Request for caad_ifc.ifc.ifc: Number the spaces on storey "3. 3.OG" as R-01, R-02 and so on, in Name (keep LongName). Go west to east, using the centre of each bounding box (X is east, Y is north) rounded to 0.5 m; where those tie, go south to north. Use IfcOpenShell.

First a look at what the model holds.

```python
import ifcopenshell
import ifcopenshell.util.element
import ifcopenshell.util.placement

model = ifcopenshell.open("caad_ifc.ifc.ifc")
print(model.schema)
storey = next(s for s in model.by_type("IfcBuildingStorey") if s.Name == "3. 3.OG")
spaces = [e for e in ifcopenshell.util.element.get_decomposition(storey) if e.is_a("IfcSpace")]
for e in sorted(spaces, key=lambda e: e.id()):
    origin = ifcopenshell.util.placement.get_local_placement(e.ObjectPlacement)[:3, 3]
    print(e.id(), e.Name, e.LongName, origin.round(2) + 0.0, sep=" | ")
```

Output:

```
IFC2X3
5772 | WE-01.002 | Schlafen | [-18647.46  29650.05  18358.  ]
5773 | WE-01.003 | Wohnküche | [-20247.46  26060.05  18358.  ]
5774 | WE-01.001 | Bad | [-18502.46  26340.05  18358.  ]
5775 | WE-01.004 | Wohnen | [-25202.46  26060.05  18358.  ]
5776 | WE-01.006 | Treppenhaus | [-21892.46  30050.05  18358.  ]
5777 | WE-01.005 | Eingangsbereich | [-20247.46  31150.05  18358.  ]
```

```python
import ifcopenshell
import ifcopenshell.geom
import ifcopenshell.util.element
import ifcopenshell.util.shape

model = ifcopenshell.open("caad_ifc.ifc.ifc")
settings = ifcopenshell.geom.settings()
settings.set("use-world-coords", True)


def centre(element):
    shape = ifcopenshell.geom.create_shape(settings, element)
    return ifcopenshell.util.shape.get_bbox_centroid(shape.geometry)


storey = next(s for s in model.by_type("IfcBuildingStorey") if s.Name == "3. 3.OG")
spaces = [e for e in ifcopenshell.util.element.get_decomposition(storey) if e.is_a("IfcSpace")]

# Insertion points can sit at a corner or the storey origin, so sort by the geometry (in metres).
centres = {e: centre(e) for e in spaces}
spaces.sort(key=lambda e: (round(centres[e][0] / 0.5), centres[e][1]))

for i, e in enumerate(spaces, start=1):
    number = f"R-{i:02d}"
    e.Name = number
    print(e.id(), number)

model.write("caad_ifc.ifc_edited.ifc")
```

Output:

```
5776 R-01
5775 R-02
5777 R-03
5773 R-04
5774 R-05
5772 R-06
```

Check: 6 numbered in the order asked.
